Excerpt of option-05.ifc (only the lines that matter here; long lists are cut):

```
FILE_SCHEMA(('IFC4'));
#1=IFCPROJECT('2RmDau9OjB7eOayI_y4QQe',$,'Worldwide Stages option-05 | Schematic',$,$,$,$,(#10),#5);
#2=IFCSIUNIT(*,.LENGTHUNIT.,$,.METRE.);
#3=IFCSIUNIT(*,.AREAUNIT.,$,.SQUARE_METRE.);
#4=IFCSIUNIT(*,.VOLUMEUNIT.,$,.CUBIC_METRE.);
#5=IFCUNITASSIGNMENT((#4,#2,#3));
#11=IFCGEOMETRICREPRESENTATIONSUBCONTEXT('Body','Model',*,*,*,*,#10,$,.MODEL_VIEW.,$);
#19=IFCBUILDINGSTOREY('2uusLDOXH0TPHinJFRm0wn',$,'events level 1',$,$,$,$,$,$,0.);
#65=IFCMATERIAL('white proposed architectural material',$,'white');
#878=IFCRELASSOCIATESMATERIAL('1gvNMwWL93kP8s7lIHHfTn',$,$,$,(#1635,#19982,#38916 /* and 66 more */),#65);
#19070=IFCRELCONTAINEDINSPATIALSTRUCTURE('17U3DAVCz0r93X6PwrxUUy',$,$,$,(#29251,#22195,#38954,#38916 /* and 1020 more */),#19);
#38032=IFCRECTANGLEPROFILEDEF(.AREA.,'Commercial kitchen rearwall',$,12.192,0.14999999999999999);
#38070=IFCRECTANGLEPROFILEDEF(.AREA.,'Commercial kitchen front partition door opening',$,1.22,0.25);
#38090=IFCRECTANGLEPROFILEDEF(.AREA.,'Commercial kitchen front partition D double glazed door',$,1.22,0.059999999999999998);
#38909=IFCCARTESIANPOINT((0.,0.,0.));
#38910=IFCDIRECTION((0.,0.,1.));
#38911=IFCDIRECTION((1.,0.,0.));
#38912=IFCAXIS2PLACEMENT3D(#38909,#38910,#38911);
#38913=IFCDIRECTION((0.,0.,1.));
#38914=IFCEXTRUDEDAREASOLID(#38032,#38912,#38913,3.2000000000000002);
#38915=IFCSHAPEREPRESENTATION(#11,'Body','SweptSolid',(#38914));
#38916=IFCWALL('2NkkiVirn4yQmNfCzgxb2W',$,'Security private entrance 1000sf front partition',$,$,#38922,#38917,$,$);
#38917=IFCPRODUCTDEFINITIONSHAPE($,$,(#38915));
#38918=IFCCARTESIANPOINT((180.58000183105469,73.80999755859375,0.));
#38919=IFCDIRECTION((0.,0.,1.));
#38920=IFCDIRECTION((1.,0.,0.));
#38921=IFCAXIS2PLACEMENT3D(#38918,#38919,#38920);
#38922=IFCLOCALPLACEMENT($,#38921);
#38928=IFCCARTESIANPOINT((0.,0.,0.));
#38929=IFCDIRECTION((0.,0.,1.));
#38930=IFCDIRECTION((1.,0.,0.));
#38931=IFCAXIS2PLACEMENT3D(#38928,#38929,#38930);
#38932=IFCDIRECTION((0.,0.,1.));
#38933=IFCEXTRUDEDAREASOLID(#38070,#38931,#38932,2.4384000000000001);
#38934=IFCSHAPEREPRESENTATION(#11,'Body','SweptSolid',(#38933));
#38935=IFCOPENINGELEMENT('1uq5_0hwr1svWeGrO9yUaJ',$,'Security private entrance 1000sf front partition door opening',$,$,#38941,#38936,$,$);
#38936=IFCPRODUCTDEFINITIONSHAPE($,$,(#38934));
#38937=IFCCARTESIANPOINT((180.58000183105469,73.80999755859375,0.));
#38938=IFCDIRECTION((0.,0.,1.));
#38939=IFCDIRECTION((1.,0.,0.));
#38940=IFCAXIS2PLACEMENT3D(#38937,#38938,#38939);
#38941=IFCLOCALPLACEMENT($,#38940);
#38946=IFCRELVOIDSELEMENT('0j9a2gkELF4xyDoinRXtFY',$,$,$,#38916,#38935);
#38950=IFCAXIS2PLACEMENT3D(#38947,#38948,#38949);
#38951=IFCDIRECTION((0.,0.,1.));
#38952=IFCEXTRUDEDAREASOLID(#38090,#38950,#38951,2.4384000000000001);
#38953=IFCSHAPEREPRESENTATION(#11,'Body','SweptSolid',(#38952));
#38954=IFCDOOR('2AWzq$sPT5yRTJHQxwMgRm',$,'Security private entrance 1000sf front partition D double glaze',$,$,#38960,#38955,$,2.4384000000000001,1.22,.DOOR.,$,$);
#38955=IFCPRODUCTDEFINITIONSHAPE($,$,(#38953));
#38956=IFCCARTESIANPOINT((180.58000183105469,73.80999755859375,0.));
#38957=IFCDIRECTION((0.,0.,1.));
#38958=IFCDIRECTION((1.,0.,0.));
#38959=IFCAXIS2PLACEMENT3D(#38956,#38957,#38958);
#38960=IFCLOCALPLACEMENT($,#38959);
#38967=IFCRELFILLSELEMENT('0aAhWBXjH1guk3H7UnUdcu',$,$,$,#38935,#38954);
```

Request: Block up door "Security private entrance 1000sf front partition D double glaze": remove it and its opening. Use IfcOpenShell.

```python
import ifcopenshell
import ifcopenshell.api.feature
import ifcopenshell.api.root
import ifcopenshell.geom
import ifcopenshell.util.shape

model = ifcopenshell.open("option-05.ifc")
settings = ifcopenshell.geom.settings()


def volume(element):
    """Net volume in cubic metres, openings subtracted."""
    shape = ifcopenshell.geom.create_shape(settings, element)
    return ifcopenshell.util.shape.get_volume(shape.geometry)


door = model.by_id(38954)
opening = door.FillsVoids[0].RelatingOpeningElement
wall = opening.VoidsElements[0].RelatingBuildingElement
before = volume(wall)

ifcopenshell.api.root.remove_product(model, product=door)
ifcopenshell.api.feature.remove_feature(model, feature=opening)

after = volume(wall)

print(f"wall volume {before:.3f} -> {after:.3f} m3")

model.write("option-05_v2.ifc")
```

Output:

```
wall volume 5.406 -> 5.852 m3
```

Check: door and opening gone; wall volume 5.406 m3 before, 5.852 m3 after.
